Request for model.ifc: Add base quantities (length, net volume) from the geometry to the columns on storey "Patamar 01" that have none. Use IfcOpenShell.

First a look at what the model holds.

```python
import ifcopenshell
import ifcopenshell.util.element
import ifcopenshell.util.unit

model = ifcopenshell.open("model.ifc")
print(model.schema)
for unit_type in ("LENGTHUNIT", "AREAUNIT", "VOLUMEUNIT"):
    print(unit_type, ifcopenshell.util.unit.calculate_unit_scale(model, unit_type))
storey = next(s for s in model.by_type("IfcBuildingStorey") if s.Name == "Patamar 01")
columns = [e for e in ifcopenshell.util.element.get_decomposition(storey) if e.is_a("IfcColumn")]
for e in sorted(columns, key=lambda e: e.id()):
    print(e.id(), e.is_a(), e.Name, list(ifcopenshell.util.element.get_psets(e, qtos_only=True)), sep=" | ")
```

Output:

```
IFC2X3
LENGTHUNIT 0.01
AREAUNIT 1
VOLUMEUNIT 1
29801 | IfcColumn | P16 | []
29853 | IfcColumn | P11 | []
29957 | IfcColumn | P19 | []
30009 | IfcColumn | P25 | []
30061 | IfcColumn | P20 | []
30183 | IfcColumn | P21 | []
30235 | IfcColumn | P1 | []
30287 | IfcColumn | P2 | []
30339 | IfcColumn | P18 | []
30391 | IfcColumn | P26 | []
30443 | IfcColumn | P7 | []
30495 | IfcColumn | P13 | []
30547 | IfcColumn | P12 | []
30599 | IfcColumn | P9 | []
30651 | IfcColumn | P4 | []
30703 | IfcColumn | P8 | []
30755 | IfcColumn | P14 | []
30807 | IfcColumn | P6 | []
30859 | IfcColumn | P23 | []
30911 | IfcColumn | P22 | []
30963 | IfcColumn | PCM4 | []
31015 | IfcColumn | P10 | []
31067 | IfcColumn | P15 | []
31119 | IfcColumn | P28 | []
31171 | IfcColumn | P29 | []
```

```python
import ifcopenshell
import ifcopenshell.api.pset
import ifcopenshell.geom
import ifcopenshell.util.element
import ifcopenshell.util.shape
import ifcopenshell.util.unit

model = ifcopenshell.open("model.ifc")
unit_scale = ifcopenshell.util.unit.calculate_unit_scale(model)
volume_scale = ifcopenshell.util.unit.calculate_unit_scale(model, "VOLUMEUNIT")
settings = ifcopenshell.geom.settings()

storey = next(s for s in model.by_type("IfcBuildingStorey") if s.Name == "Patamar 01")
columns = [e for e in ifcopenshell.util.element.get_decomposition(storey) if e.is_a("IfcColumn")]

for e in sorted(columns, key=lambda e: e.id()):
    if ifcopenshell.util.element.get_psets(e, qtos_only=True, should_inherit=False):
        continue
    # Geometry comes back in metres, in the element's own axes.
    shape = ifcopenshell.geom.create_shape(settings, e)
    values = {
        "Length": ifcopenshell.util.shape.get_z(shape.geometry) / unit_scale,
        "NetVolume": ifcopenshell.util.shape.get_volume(shape.geometry) / volume_scale,
    }
    qto = ifcopenshell.api.pset.add_qto(model, product=e, name="BaseQuantities")
    ifcopenshell.api.pset.edit_qto(model, qto=qto, properties=values)
    print(e.id(), {k: round(v, 3) for k, v in values.items()})

model.write("model_v2.ifc")
```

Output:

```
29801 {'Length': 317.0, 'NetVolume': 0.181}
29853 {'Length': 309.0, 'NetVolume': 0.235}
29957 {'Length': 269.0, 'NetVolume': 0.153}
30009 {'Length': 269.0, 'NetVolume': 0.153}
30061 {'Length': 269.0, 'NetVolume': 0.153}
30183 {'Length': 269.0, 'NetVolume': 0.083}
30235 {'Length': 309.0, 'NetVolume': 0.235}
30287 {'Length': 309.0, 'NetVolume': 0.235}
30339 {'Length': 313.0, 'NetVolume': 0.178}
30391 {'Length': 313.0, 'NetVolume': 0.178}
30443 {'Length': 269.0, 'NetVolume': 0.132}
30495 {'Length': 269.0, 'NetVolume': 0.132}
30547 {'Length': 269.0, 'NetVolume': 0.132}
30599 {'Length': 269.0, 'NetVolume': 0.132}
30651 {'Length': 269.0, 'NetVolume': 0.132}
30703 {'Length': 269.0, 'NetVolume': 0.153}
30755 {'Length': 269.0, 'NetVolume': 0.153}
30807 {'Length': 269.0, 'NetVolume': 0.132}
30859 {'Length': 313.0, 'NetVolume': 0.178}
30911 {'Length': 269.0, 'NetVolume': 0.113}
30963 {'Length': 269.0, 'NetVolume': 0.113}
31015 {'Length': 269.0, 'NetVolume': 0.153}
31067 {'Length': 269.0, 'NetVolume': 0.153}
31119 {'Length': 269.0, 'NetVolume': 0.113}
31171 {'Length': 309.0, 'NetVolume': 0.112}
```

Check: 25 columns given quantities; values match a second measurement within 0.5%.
